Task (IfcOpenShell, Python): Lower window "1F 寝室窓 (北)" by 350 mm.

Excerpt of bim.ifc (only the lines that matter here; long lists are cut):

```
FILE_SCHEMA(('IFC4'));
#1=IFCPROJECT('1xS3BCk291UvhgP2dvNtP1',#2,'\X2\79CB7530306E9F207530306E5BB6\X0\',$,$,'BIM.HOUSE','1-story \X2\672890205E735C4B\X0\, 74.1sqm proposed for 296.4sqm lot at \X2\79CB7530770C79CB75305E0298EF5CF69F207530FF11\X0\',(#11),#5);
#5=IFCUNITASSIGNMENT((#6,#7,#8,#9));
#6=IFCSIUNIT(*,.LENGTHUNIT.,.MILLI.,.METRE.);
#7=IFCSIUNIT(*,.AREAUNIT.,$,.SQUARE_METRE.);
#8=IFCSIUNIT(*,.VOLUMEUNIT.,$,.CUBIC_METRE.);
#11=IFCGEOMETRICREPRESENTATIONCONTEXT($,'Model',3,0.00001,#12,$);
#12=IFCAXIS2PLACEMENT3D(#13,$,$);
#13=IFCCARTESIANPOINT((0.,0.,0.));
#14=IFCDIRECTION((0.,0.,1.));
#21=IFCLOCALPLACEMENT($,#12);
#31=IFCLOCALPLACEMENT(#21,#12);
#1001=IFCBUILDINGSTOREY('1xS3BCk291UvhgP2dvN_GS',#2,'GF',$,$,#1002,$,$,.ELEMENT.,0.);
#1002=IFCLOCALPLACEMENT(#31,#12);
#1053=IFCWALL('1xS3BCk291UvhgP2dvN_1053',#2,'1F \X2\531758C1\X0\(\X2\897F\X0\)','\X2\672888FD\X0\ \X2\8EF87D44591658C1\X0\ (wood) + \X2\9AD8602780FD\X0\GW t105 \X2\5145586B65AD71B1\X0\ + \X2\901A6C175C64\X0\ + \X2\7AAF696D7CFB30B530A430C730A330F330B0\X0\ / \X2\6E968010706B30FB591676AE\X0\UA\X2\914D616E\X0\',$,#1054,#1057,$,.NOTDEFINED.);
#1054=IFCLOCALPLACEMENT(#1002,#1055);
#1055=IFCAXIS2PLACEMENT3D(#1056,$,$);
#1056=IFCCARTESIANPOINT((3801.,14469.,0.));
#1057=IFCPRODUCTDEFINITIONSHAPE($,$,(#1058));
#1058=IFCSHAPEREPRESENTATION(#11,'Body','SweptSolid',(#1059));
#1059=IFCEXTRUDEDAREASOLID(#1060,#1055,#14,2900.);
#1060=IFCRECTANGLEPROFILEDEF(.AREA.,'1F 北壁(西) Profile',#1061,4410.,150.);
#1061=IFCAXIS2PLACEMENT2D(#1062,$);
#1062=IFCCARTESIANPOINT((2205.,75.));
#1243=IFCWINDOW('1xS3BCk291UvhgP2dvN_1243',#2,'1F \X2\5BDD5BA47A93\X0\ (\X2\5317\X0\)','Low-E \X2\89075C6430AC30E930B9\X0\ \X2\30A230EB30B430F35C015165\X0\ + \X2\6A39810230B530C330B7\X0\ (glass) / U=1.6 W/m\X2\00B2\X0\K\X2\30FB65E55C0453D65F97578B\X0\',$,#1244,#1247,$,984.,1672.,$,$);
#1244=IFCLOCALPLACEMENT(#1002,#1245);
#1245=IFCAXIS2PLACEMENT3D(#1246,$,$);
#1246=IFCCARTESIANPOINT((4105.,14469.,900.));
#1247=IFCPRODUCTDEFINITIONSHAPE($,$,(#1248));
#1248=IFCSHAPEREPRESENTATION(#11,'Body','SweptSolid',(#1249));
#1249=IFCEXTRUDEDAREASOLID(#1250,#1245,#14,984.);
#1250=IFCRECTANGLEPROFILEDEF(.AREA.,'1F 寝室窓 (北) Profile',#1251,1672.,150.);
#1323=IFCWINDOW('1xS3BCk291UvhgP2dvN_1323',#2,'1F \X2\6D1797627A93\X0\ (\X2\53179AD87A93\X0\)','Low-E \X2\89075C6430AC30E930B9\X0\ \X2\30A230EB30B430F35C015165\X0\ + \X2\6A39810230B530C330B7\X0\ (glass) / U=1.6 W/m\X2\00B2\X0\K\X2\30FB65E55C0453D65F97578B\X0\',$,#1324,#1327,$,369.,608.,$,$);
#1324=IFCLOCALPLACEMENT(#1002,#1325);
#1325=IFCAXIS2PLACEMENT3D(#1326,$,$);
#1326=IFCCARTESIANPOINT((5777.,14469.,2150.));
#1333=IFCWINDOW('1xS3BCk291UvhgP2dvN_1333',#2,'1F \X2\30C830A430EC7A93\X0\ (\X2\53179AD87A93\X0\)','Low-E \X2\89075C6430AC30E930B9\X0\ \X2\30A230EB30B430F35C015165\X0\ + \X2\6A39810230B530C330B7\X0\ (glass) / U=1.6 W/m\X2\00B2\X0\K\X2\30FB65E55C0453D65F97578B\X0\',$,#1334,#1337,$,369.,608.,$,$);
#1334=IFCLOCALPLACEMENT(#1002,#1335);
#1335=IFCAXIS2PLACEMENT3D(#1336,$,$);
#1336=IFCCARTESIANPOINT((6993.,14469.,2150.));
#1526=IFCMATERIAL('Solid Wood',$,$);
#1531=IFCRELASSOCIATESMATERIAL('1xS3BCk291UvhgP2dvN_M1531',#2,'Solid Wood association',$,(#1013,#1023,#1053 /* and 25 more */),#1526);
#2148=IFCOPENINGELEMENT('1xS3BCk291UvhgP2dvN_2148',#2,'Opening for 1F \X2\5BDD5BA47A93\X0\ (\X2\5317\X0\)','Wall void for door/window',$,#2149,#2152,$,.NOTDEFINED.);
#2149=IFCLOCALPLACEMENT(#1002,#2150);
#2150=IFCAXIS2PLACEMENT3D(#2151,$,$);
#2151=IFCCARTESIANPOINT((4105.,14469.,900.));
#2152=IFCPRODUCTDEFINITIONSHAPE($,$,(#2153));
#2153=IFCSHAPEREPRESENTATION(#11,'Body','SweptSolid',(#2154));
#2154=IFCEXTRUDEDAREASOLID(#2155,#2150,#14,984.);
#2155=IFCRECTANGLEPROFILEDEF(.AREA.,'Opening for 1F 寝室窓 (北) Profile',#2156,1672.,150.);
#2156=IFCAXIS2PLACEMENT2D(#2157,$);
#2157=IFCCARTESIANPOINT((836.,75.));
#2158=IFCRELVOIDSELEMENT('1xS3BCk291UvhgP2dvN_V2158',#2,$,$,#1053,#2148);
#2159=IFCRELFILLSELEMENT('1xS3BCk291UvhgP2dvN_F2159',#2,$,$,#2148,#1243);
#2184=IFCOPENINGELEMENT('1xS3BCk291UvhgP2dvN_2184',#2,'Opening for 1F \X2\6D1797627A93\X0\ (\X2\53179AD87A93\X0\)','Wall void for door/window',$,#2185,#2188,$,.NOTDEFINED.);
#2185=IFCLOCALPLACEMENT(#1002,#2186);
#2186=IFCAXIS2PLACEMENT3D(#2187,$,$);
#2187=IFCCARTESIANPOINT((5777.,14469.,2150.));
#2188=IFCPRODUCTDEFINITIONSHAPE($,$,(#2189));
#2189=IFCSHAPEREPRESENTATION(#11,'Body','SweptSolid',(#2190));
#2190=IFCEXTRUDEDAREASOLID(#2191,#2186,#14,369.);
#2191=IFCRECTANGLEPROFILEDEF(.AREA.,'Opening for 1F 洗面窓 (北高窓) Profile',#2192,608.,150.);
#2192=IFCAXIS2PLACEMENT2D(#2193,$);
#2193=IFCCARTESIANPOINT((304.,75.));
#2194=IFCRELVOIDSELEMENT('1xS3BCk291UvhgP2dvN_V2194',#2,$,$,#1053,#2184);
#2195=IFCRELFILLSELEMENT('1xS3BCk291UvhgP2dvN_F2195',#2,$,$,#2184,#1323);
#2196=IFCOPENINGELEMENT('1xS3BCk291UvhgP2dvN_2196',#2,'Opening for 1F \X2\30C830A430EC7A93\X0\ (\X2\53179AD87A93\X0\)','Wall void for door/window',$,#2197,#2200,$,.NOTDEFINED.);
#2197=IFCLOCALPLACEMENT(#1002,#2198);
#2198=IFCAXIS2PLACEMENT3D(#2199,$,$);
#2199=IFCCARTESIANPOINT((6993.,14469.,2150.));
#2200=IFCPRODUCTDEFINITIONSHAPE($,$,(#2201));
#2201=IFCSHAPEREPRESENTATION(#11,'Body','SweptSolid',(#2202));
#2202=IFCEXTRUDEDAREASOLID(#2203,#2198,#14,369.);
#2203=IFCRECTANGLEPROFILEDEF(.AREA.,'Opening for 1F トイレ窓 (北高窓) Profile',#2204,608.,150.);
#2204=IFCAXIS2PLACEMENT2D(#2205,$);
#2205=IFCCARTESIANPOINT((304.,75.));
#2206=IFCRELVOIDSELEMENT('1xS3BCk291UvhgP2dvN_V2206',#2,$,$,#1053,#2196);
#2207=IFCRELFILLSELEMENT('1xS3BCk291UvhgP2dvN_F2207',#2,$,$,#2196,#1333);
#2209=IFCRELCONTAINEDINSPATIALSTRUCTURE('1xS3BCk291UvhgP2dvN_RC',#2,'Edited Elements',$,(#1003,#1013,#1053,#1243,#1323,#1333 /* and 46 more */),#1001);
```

```python
import numpy as np
import ifcopenshell
import ifcopenshell.api.geometry
import ifcopenshell.util.placement
import ifcopenshell.util.unit

model = ifcopenshell.open("bim.ifc")
unit_scale = ifcopenshell.util.unit.calculate_unit_scale(model)

window = model.by_id(1243)
opening = window.FillsVoids[0].RelatingOpeningElement
dz = -350.0

shift = np.array([0.0, 0.0, dz])
# The window is not placed relative to its opening, so move both.
for product in (opening, window):
    matrix = ifcopenshell.util.placement.get_local_placement(product.ObjectPlacement)
    matrix[:3, 3] += shift
    ifcopenshell.api.geometry.edit_object_placement(model, product=product, matrix=matrix, is_si=False)

print(f"moved by {dz * unit_scale:+.3f} m")

model.write("bim-out.ifc")
```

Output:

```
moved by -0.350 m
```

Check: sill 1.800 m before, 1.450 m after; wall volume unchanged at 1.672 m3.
